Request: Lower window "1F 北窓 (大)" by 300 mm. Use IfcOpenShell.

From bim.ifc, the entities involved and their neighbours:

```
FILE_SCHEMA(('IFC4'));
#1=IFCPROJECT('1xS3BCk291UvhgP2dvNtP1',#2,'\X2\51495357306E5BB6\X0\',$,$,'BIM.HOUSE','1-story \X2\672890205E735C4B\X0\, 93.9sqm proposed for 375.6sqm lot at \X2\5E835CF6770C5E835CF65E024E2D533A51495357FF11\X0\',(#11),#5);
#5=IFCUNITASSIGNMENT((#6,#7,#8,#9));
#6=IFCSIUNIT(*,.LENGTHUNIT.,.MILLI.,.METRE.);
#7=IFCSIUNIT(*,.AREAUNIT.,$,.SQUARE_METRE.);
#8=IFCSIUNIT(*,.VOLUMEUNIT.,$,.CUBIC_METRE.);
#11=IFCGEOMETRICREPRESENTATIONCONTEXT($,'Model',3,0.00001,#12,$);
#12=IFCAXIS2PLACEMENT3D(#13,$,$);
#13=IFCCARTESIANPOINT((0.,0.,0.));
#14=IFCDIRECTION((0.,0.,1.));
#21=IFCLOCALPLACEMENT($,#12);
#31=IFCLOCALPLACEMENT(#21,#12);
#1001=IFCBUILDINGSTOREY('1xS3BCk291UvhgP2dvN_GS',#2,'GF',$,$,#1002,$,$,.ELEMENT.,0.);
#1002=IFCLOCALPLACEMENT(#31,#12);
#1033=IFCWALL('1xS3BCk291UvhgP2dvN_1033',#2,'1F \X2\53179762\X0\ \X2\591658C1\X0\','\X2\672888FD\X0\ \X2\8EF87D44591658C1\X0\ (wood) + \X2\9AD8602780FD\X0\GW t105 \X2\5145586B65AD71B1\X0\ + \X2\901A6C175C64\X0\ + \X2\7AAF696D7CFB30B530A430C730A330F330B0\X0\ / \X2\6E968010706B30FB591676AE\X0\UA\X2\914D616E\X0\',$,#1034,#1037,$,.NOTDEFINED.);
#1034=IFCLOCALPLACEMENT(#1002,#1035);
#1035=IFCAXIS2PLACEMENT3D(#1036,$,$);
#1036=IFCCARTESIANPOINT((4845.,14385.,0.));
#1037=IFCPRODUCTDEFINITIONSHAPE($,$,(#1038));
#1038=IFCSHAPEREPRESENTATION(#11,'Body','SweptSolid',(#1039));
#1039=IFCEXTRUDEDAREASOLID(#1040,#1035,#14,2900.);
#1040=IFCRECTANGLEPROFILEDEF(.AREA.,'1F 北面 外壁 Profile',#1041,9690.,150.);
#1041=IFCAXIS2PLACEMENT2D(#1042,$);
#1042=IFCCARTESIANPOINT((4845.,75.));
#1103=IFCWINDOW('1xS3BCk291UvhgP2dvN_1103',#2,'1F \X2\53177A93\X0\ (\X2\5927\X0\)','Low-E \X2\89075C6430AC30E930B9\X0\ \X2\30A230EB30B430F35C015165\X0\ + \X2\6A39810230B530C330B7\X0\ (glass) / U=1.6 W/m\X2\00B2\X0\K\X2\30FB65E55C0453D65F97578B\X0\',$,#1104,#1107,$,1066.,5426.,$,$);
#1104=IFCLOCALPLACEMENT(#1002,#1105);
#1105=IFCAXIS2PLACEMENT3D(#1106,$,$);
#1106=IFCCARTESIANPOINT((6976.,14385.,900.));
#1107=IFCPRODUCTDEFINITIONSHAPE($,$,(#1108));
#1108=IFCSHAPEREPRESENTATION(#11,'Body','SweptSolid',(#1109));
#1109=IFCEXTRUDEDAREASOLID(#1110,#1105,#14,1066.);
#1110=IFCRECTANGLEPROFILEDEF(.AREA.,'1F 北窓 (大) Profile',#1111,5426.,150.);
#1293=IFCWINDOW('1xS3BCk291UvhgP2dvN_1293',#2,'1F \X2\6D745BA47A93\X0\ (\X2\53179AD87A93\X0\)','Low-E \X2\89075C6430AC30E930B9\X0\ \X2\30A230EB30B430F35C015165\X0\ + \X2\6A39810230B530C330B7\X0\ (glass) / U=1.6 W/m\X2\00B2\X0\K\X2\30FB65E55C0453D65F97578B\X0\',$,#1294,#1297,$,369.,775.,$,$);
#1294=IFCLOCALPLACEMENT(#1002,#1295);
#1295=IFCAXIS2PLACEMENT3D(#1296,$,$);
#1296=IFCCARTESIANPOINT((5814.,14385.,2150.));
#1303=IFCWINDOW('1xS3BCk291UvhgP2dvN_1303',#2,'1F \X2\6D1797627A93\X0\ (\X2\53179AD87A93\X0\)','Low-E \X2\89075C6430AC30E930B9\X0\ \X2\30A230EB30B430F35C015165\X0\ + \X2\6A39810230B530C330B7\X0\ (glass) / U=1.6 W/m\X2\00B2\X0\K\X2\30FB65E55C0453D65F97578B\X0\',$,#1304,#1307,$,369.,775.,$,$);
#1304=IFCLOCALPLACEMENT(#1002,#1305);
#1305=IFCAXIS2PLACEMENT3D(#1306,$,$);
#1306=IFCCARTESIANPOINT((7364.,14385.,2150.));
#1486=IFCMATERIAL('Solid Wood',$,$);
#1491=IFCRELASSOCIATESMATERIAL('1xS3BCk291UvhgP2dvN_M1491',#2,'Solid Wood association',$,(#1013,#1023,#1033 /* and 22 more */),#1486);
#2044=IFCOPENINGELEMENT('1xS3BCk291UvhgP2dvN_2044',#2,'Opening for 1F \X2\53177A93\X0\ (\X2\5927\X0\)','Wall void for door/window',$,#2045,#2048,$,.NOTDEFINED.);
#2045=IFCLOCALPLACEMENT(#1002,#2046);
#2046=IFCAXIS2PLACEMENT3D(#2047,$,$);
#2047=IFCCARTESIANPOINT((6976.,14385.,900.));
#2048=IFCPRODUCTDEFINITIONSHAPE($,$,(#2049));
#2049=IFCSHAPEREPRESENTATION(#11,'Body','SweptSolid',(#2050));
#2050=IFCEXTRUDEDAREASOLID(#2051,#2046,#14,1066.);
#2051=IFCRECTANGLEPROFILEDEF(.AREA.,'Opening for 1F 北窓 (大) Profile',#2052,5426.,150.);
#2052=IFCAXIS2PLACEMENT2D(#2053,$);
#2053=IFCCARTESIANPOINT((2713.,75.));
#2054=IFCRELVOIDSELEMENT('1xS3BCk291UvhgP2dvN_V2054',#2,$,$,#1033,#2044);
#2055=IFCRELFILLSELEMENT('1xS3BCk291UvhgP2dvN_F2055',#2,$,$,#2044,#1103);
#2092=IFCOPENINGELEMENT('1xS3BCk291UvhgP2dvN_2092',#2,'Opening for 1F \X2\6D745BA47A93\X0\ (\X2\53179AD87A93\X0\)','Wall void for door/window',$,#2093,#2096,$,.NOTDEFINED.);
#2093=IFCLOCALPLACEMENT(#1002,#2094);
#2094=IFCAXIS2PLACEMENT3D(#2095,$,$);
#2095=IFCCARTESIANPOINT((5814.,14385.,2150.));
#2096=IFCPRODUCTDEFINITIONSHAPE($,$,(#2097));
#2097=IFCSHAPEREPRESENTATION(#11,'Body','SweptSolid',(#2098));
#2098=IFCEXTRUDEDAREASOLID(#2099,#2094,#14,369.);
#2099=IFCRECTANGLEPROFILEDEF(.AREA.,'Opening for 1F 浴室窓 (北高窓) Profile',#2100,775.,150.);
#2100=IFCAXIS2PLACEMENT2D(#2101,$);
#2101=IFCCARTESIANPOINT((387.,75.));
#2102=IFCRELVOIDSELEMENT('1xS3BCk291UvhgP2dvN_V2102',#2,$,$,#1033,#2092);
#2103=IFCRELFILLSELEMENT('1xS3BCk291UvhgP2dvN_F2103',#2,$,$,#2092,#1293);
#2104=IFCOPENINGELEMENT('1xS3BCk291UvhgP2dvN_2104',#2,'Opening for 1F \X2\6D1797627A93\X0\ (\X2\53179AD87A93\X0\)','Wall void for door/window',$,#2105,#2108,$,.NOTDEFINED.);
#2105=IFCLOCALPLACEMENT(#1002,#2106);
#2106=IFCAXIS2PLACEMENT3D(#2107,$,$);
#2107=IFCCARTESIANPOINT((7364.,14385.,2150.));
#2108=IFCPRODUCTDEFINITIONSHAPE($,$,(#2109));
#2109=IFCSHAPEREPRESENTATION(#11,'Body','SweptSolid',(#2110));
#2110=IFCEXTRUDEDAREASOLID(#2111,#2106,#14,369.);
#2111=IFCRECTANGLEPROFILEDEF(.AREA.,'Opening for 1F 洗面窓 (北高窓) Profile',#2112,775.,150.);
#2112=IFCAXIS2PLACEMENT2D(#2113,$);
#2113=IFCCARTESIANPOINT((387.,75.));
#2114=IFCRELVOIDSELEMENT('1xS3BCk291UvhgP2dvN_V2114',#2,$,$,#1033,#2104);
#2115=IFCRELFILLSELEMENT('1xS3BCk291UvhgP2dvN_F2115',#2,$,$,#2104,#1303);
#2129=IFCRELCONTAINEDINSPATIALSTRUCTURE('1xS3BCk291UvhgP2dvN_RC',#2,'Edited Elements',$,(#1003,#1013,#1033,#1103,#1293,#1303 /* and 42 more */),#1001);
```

```python
import numpy as np
import ifcopenshell
import ifcopenshell.api.geometry
import ifcopenshell.util.placement
import ifcopenshell.util.unit

model = ifcopenshell.open("bim.ifc")
unit_scale = ifcopenshell.util.unit.calculate_unit_scale(model)

window = model.by_id(1103)
opening = window.FillsVoids[0].RelatingOpeningElement
dz = -0.3 / unit_scale

shift = np.array([0.0, 0.0, dz])
# The window is not placed relative to its opening, so move both.
for product in (opening, window):
    matrix = ifcopenshell.util.placement.get_local_placement(product.ObjectPlacement)
    matrix[:3, 3] += shift
    ifcopenshell.api.geometry.edit_object_placement(model, product=product, matrix=matrix, is_si=False)

print(f"moved by {dz * unit_scale:+.3f} m")

model.write("bim-out.ifc")
```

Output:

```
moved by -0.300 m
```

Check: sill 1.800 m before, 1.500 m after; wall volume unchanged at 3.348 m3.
